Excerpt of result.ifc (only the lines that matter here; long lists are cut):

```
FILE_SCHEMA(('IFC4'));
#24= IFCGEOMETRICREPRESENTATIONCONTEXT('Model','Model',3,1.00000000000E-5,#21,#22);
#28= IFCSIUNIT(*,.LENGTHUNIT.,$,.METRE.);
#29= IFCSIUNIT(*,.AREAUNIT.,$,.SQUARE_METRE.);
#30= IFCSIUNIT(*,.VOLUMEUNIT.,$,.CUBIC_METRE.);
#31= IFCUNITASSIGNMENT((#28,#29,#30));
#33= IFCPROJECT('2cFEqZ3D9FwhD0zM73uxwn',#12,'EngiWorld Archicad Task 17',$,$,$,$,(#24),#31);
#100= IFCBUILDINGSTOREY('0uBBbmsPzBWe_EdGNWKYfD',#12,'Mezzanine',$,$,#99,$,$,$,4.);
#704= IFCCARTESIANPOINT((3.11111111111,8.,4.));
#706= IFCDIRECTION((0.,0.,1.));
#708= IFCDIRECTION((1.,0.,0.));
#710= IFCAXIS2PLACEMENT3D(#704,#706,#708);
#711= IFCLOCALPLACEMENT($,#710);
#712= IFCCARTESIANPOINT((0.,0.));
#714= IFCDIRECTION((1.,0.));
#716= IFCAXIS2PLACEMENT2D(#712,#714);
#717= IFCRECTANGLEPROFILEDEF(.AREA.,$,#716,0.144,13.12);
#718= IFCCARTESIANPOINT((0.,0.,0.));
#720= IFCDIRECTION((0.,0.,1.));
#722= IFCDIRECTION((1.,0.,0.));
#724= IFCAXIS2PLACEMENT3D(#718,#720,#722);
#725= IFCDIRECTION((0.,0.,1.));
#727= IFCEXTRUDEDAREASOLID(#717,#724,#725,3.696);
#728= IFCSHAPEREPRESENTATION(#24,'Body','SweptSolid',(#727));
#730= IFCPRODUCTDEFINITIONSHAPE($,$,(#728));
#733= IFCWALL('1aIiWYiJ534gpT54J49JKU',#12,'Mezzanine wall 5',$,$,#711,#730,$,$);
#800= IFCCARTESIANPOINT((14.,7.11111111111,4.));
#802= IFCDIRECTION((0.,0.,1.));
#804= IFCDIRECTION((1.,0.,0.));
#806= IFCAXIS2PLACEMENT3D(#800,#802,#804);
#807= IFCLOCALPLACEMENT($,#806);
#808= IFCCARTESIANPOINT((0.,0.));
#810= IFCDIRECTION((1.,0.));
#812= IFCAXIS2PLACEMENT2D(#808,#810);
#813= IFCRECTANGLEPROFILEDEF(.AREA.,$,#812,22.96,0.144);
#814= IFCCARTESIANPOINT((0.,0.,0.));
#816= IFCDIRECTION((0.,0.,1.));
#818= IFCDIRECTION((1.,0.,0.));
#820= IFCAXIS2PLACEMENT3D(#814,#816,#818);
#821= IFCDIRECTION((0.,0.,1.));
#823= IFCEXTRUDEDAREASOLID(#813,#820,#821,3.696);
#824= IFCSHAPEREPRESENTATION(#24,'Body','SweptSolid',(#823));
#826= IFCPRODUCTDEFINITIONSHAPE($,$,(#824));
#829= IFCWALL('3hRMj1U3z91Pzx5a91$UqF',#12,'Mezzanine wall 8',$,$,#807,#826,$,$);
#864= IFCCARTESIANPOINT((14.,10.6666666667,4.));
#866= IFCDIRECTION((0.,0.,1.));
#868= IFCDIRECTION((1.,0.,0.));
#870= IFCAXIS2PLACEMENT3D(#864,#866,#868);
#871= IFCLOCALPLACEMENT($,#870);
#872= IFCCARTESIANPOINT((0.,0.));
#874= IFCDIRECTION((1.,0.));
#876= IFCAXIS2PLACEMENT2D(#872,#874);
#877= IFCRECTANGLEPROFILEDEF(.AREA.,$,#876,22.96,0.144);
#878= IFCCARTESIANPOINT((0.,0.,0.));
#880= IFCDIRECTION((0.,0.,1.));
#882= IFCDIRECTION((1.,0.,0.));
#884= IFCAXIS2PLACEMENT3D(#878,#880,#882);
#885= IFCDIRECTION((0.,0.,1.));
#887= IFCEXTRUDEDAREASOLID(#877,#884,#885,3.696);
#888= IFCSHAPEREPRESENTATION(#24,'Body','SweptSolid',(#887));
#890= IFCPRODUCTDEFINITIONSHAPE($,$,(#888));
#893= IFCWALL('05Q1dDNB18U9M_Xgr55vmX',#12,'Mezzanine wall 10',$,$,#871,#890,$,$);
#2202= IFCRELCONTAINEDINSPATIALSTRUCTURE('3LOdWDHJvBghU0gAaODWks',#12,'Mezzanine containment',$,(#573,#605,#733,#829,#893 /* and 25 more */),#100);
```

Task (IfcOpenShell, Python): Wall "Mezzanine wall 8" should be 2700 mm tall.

```python
import ifcopenshell
import ifcopenshell.geom
import ifcopenshell.util.shape
import ifcopenshell.util.unit

model = ifcopenshell.open("result.ifc")
unit_scale = ifcopenshell.util.unit.calculate_unit_scale(model)
settings = ifcopenshell.geom.settings()


def volume(element):
    """Net volume in cubic metres, openings subtracted."""
    shape = ifcopenshell.geom.create_shape(settings, element)
    return ifcopenshell.util.shape.get_volume(shape.geometry)


wall = model.by_id(829)
before = volume(wall)

body = next(r for r in wall.Representation.Representations if r.RepresentationIdentifier == "Body")
solid = body.Items[0]
old_height = solid.Depth
solid.Depth = 2.7 / unit_scale
after = volume(wall)

print(f"height {old_height:g} -> {solid.Depth:g}, volume {before:.3f} -> {after:.3f} m3")

model.write("result_rev.ifc")
```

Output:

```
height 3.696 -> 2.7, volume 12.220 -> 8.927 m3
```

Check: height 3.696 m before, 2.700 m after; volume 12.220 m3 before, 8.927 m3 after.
